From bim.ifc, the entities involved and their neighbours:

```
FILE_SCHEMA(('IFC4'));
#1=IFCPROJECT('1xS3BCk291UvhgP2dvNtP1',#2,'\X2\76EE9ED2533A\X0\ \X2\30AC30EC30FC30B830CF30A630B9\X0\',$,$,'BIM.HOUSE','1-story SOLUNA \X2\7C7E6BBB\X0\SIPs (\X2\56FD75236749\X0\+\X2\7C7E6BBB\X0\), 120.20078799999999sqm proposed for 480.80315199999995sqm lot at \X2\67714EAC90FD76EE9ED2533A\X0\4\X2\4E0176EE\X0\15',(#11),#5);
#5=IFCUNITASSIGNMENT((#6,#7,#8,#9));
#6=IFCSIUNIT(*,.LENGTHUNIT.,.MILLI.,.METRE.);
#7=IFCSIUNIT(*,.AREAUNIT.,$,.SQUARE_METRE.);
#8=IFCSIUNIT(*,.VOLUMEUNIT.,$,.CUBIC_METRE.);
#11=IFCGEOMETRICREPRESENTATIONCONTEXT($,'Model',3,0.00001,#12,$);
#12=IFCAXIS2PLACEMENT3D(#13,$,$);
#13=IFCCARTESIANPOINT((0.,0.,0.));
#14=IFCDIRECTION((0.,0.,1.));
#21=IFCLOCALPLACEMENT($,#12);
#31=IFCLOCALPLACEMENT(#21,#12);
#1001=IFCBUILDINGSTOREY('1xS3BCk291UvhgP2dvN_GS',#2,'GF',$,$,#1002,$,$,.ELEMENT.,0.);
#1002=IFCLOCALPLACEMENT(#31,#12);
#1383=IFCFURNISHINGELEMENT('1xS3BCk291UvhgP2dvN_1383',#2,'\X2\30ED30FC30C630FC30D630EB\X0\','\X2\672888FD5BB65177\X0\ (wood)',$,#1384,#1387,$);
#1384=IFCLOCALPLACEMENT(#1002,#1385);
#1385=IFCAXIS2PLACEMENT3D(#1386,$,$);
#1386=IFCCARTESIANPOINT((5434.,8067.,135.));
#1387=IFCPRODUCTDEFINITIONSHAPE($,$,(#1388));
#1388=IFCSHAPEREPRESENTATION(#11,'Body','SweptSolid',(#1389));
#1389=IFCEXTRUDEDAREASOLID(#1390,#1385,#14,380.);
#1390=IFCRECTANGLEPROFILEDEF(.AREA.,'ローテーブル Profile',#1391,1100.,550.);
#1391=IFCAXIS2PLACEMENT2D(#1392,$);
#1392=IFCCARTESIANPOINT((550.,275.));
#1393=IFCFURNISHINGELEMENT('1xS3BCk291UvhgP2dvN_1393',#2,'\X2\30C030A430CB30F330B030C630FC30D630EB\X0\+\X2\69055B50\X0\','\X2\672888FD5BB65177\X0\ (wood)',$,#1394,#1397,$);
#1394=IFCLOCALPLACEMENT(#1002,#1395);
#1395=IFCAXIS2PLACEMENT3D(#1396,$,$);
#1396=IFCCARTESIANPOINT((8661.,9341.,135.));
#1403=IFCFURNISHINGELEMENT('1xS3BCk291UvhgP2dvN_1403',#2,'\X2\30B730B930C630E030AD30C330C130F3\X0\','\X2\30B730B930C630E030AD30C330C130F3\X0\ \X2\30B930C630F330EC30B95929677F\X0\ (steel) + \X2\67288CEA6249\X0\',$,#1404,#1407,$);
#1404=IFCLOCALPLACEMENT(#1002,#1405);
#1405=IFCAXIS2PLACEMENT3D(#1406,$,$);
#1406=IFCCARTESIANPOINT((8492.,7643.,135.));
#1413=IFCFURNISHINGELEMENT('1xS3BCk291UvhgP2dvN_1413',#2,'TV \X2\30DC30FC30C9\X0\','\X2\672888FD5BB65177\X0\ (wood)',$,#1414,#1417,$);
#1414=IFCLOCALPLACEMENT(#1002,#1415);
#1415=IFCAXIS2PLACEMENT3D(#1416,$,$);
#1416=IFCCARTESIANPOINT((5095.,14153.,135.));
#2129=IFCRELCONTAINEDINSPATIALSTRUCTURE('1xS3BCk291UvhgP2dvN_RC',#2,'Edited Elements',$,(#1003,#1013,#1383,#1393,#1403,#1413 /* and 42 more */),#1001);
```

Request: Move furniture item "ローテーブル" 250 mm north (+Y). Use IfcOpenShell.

```python
import ifcopenshell
import ifcopenshell.api.geometry
import ifcopenshell.util.placement
import ifcopenshell.util.unit

model = ifcopenshell.open("bim.ifc")
unit_scale = ifcopenshell.util.unit.calculate_unit_scale(model)

item = model.by_id(1383)
matrix = ifcopenshell.util.placement.get_local_placement(item.ObjectPlacement)
matrix[1, 3] += 0.25 / unit_scale
ifcopenshell.api.geometry.edit_object_placement(model, product=item, matrix=matrix, is_si=False)

print(ifcopenshell.util.placement.get_local_placement(item.ObjectPlacement).round(3) + 0.0)

model.write("bim_v2.ifc")
```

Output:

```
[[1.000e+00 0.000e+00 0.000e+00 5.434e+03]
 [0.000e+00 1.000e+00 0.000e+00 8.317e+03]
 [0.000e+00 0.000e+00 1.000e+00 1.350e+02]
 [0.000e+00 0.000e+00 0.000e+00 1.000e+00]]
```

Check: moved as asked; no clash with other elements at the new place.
